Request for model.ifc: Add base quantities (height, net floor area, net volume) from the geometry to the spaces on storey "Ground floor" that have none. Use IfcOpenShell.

First a look at what the model holds.

```python
import ifcopenshell
import ifcopenshell.util.element
import ifcopenshell.util.unit

model = ifcopenshell.open("model.ifc")
print(model.schema)
for unit_type in ("LENGTHUNIT", "AREAUNIT", "VOLUMEUNIT"):
    print(unit_type, ifcopenshell.util.unit.calculate_unit_scale(model, unit_type))
storey = next(s for s in model.by_type("IfcBuildingStorey") if s.Name == "Ground floor")
spaces = [e for e in ifcopenshell.util.element.get_decomposition(storey) if e.is_a("IfcSpace")]
for e in sorted(spaces, key=lambda e: e.id()):
    print(e.id(), e.is_a(), e.Name, list(ifcopenshell.util.element.get_psets(e, qtos_only=True)), sep=" | ")
```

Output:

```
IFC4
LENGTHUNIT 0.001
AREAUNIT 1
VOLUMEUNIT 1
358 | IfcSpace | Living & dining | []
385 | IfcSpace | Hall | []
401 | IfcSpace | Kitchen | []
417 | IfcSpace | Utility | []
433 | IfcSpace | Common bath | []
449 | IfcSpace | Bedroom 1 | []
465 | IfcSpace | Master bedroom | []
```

```python
import ifcopenshell
import ifcopenshell.api.pset
import ifcopenshell.geom
import ifcopenshell.util.element
import ifcopenshell.util.shape
import ifcopenshell.util.unit

model = ifcopenshell.open("model.ifc")
unit_scale = ifcopenshell.util.unit.calculate_unit_scale(model)
area_scale = ifcopenshell.util.unit.calculate_unit_scale(model, "AREAUNIT")
volume_scale = ifcopenshell.util.unit.calculate_unit_scale(model, "VOLUMEUNIT")
settings = ifcopenshell.geom.settings()

storey = next(s for s in model.by_type("IfcBuildingStorey") if s.Name == "Ground floor")
spaces = [e for e in ifcopenshell.util.element.get_decomposition(storey) if e.is_a("IfcSpace")]

for e in sorted(spaces, key=lambda e: e.id()):
    if ifcopenshell.util.element.get_psets(e, qtos_only=True, should_inherit=False):
        continue
    # Geometry comes back in metres, in the element's own axes.
    shape = ifcopenshell.geom.create_shape(settings, e)
    values = {
        "Height": ifcopenshell.util.shape.get_z(shape.geometry) / unit_scale,
        "NetFloorArea": ifcopenshell.util.shape.get_footprint_area(shape.geometry) / area_scale,
        "NetVolume": ifcopenshell.util.shape.get_volume(shape.geometry) / volume_scale,
    }
    qto = ifcopenshell.api.pset.add_qto(model, product=e, name="Qto_SpaceBaseQuantities")
    ifcopenshell.api.pset.edit_qto(model, qto=qto, properties=values)
    print(e.id(), {k: round(v, 3) for k, v in values.items()})

model.write("model_edited.ifc")
```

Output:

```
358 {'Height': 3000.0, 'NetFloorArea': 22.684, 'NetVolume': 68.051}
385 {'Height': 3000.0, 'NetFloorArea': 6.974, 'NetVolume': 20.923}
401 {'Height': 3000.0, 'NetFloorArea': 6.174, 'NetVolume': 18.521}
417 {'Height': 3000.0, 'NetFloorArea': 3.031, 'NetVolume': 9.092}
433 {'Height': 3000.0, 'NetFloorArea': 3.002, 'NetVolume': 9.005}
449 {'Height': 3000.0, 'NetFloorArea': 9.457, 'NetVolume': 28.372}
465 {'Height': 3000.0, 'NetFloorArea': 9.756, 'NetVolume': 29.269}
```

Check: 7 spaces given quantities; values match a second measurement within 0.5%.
